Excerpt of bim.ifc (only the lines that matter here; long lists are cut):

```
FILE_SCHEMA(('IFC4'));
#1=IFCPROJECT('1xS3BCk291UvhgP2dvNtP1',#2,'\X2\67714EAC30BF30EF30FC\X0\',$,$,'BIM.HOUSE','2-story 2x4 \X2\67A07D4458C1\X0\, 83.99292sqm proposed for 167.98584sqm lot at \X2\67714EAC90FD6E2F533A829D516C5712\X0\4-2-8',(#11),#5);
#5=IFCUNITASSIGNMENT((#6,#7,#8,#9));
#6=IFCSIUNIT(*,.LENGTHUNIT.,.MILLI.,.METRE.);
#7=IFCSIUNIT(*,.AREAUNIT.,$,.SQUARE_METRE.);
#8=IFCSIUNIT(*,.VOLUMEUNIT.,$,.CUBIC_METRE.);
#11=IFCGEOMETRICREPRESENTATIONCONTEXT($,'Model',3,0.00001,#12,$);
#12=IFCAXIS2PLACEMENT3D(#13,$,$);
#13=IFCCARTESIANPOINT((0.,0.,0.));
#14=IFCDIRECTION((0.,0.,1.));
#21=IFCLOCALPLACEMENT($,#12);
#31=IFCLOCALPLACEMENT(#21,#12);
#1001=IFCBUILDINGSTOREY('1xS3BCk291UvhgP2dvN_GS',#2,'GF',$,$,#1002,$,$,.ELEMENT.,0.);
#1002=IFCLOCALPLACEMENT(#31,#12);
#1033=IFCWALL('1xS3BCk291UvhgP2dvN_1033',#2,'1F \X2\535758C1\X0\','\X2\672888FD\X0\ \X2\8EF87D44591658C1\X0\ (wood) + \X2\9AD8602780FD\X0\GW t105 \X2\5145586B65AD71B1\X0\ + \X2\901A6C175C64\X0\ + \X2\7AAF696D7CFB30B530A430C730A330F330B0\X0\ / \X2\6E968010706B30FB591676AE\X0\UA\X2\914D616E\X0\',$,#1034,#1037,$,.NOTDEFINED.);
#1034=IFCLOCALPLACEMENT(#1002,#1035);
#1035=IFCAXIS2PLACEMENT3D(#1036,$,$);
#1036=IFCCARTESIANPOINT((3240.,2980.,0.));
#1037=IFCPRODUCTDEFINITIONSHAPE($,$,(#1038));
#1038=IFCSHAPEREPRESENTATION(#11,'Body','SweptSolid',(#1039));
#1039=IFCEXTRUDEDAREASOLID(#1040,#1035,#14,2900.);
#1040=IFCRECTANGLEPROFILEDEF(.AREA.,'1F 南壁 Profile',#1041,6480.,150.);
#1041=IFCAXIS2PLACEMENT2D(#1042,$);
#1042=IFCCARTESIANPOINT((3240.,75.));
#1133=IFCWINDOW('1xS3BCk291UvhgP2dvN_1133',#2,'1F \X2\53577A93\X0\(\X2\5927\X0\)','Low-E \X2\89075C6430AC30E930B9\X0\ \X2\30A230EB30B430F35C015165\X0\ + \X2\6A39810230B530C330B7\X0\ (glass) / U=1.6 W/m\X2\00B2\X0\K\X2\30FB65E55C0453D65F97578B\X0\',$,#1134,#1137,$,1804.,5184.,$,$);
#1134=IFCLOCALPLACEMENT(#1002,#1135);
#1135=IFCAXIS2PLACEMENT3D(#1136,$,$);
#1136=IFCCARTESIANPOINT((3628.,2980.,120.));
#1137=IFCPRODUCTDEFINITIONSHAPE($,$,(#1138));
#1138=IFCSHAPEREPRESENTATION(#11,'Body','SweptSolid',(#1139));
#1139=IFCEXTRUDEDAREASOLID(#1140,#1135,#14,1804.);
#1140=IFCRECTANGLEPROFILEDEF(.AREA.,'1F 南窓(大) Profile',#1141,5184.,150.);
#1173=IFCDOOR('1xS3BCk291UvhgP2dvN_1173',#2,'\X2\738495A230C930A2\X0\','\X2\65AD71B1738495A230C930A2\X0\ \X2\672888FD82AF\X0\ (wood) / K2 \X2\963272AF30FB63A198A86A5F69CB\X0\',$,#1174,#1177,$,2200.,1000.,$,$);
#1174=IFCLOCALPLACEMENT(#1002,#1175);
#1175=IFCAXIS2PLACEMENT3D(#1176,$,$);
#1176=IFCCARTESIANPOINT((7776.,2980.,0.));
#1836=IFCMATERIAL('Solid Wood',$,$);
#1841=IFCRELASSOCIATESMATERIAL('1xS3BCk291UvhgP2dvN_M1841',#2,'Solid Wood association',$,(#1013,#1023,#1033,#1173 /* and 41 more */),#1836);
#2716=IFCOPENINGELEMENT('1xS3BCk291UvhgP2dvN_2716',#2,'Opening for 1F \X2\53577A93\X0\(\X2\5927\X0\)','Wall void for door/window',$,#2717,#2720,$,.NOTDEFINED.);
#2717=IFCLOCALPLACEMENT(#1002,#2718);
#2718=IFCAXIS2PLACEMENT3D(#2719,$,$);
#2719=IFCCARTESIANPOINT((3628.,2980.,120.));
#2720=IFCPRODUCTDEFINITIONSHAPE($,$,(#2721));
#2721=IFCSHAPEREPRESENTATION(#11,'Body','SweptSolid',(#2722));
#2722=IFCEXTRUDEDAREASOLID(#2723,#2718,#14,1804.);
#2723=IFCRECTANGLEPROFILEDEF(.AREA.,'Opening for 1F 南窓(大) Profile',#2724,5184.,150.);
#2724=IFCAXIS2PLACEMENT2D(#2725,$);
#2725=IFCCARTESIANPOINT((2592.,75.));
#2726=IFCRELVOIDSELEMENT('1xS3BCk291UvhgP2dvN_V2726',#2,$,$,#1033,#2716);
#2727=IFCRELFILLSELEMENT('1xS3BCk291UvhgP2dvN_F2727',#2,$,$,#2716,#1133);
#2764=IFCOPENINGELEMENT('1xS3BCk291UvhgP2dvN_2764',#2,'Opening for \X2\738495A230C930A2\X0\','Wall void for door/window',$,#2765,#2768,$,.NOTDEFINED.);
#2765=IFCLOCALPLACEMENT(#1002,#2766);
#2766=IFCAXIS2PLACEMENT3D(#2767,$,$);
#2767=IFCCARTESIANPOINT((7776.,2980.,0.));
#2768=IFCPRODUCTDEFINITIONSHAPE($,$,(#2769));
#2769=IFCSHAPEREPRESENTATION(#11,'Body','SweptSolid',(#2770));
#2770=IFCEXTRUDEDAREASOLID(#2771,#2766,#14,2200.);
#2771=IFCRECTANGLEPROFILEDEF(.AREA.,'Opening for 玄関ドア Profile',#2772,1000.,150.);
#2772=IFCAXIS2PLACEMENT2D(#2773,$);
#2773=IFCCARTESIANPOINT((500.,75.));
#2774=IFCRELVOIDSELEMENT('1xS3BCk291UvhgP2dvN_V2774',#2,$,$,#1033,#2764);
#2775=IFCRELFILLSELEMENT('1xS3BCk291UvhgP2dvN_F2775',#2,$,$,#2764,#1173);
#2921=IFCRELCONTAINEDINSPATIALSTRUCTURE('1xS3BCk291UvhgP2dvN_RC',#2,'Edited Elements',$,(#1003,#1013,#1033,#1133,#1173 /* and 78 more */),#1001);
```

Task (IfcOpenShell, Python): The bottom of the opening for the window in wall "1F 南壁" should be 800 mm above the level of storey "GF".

```python
import numpy as np
import ifcopenshell
import ifcopenshell.api.geometry
import ifcopenshell.geom
import ifcopenshell.util.element
import ifcopenshell.util.placement
import ifcopenshell.util.shape
import ifcopenshell.util.unit

model = ifcopenshell.open("bim.ifc")
unit_scale = ifcopenshell.util.unit.calculate_unit_scale(model)

window = model.by_id(1133)
opening = window.FillsVoids[0].RelatingOpeningElement
storey = ifcopenshell.util.element.get_container(window, ifc_class="IfcBuildingStorey")
level = ifcopenshell.util.placement.get_local_placement(storey.ObjectPlacement)[2, 3]

# The opening's origin need not be at the sill, so measure its lowest point.
shape = ifcopenshell.geom.create_shape(ifcopenshell.geom.settings(), opening)
bottom = ifcopenshell.util.shape.get_shape_bottom_elevation(shape, shape.geometry) / unit_scale
dz = level + 800.0 - bottom

shift = np.array([0.0, 0.0, dz])
# The window is not placed relative to its opening, so move both.
for product in (opening, window):
    matrix = ifcopenshell.util.placement.get_local_placement(product.ObjectPlacement)
    matrix[:3, 3] += shift
    ifcopenshell.api.geometry.edit_object_placement(model, product=product, matrix=matrix, is_si=False)

print(f"moved by {dz * unit_scale:+.3f} m")

model.write("bim-out.ifc")
```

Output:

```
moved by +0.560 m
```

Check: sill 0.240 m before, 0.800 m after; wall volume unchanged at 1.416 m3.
